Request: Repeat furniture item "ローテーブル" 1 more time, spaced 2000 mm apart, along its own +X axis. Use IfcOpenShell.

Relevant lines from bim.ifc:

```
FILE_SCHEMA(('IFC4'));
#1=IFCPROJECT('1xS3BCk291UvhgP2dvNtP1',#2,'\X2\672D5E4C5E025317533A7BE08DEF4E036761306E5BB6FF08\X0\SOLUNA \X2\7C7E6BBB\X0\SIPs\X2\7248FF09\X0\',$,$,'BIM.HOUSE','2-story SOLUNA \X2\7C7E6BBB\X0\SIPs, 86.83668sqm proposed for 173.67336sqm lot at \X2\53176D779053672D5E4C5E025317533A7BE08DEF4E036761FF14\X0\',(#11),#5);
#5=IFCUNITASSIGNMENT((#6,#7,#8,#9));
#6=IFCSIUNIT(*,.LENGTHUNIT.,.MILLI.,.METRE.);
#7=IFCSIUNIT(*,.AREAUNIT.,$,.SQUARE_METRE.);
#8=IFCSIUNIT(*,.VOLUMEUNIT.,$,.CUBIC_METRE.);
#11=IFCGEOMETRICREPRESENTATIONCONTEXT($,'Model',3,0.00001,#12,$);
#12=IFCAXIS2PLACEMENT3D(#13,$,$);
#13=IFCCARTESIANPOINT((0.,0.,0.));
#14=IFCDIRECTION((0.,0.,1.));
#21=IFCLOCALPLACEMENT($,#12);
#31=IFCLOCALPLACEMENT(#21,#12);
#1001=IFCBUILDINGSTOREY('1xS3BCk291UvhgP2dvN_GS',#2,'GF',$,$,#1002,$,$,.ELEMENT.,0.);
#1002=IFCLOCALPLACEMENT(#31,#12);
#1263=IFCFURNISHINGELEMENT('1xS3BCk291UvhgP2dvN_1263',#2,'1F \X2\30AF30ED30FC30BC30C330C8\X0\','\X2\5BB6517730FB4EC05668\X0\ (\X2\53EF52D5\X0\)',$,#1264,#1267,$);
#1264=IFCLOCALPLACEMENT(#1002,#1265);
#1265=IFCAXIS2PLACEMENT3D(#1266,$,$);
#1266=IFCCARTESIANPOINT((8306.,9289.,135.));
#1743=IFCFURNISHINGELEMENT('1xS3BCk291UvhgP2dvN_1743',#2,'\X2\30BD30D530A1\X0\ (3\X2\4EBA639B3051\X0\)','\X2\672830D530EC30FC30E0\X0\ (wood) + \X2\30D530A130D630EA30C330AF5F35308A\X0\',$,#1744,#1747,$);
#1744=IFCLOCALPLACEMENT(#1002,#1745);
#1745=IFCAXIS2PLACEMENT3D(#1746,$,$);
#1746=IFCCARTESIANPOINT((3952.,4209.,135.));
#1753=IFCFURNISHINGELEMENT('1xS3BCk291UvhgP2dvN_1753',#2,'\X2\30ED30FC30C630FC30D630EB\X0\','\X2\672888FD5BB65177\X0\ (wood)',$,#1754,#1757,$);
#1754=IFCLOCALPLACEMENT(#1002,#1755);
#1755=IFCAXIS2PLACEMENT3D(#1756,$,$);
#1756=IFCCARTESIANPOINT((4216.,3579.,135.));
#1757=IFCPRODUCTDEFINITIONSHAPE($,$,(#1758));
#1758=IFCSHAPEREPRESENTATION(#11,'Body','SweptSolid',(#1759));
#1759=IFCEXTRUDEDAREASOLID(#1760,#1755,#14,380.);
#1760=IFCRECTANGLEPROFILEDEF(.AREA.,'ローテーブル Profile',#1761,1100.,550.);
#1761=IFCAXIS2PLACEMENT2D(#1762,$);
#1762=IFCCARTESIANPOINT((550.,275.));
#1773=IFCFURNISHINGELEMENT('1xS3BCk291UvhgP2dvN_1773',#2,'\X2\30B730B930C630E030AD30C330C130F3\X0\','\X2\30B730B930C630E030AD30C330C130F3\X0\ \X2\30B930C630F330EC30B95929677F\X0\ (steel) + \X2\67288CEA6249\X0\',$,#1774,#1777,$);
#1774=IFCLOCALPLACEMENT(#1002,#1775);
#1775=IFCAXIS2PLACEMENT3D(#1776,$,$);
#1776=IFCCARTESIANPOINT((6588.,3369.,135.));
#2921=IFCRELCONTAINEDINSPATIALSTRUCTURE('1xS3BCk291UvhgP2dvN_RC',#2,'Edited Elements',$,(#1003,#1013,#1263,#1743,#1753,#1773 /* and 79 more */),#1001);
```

```python
import ifcopenshell
import ifcopenshell.api.geometry
import ifcopenshell.api.root
import ifcopenshell.util.element
import ifcopenshell.util.placement

model = ifcopenshell.open("bim.ifc")


def reuse_history(source, copy):
    """copy_class also copies each property set's owner history, people and application; keep the originals."""
    for rel in copy.IsDefinedBy:
        if rel.is_a("IfcRelDefinesByProperties") and (history := rel.RelatingPropertyDefinition.OwnerHistory):
            rel.RelatingPropertyDefinition.OwnerHistory = source.OwnerHistory
            ifcopenshell.util.element.remove_deep2(model, history)


source = model.by_id(1753)
base = ifcopenshell.util.placement.get_local_placement(source.ObjectPlacement)
step = base[:3, 0] * 2000.0

for i in range(1, 2):
    copy = ifcopenshell.api.root.copy_class(model, product=source)
    copy.Representation = ifcopenshell.util.element.copy_deep(
        model, source.Representation, exclude=["IfcGeometricRepresentationContext", "IfcRepresentationMap"]
    )
    reuse_history(source, copy)
    matrix = base.copy()
    matrix[:3, 3] += i * step
    print("added at", matrix[:3, 3].round(3) + 0.0)
    ifcopenshell.api.geometry.edit_object_placement(model, product=copy, matrix=matrix, is_si=False)

model.write("bim_rev.ifc")
```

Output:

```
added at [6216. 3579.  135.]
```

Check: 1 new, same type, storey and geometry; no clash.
